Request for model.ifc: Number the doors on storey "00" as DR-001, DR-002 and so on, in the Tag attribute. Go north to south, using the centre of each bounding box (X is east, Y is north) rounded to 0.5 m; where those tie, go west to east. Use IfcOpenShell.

First a look at what the model holds.

```python
import ifcopenshell
import ifcopenshell.util.element
import ifcopenshell.util.placement

model = ifcopenshell.open("model.ifc")
print(model.schema)
storey = next(s for s in model.by_type("IfcBuildingStorey") if s.Name == "00")
doors = [e for e in ifcopenshell.util.element.get_decomposition(storey) if e.is_a("IfcDoor")]
for e in sorted(doors, key=lambda e: e.id()):
    origin = ifcopenshell.util.placement.get_local_placement(e.ObjectPlacement)[:3, 3]
    print(e.id(), e.Tag, e.Name, origin.round(2) + 0.0, sep=" | ")
```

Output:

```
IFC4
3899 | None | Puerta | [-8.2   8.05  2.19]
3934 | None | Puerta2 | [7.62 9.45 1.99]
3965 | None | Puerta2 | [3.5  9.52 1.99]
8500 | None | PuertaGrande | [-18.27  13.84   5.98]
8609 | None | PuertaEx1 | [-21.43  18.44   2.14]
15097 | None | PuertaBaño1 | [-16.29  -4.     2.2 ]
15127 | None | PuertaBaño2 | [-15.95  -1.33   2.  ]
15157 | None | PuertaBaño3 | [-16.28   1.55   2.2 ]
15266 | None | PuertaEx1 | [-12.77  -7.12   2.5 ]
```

```python
import ifcopenshell
import ifcopenshell.geom
import ifcopenshell.util.element
import ifcopenshell.util.shape

model = ifcopenshell.open("model.ifc")
settings = ifcopenshell.geom.settings()
settings.set("use-world-coords", True)


def centre(element):
    shape = ifcopenshell.geom.create_shape(settings, element)
    return ifcopenshell.util.shape.get_bbox_centroid(shape.geometry)


storey = next(s for s in model.by_type("IfcBuildingStorey") if s.Name == "00")
doors = [e for e in ifcopenshell.util.element.get_decomposition(storey) if e.is_a("IfcDoor")]

# Insertion points can sit at a corner or the storey origin, so sort by the geometry (in metres).
centres = {e: centre(e) for e in doors}
doors.sort(key=lambda e: (-round(centres[e][1] / 0.5), centres[e][0]))

for i, e in enumerate(doors, start=1):
    number = f"DR-0{i:02d}"
    e.Tag = number
    print(e.id(), number)

model.write("model-out.ifc")
```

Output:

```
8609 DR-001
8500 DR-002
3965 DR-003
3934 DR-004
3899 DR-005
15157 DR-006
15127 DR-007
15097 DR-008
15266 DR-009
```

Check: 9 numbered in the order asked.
